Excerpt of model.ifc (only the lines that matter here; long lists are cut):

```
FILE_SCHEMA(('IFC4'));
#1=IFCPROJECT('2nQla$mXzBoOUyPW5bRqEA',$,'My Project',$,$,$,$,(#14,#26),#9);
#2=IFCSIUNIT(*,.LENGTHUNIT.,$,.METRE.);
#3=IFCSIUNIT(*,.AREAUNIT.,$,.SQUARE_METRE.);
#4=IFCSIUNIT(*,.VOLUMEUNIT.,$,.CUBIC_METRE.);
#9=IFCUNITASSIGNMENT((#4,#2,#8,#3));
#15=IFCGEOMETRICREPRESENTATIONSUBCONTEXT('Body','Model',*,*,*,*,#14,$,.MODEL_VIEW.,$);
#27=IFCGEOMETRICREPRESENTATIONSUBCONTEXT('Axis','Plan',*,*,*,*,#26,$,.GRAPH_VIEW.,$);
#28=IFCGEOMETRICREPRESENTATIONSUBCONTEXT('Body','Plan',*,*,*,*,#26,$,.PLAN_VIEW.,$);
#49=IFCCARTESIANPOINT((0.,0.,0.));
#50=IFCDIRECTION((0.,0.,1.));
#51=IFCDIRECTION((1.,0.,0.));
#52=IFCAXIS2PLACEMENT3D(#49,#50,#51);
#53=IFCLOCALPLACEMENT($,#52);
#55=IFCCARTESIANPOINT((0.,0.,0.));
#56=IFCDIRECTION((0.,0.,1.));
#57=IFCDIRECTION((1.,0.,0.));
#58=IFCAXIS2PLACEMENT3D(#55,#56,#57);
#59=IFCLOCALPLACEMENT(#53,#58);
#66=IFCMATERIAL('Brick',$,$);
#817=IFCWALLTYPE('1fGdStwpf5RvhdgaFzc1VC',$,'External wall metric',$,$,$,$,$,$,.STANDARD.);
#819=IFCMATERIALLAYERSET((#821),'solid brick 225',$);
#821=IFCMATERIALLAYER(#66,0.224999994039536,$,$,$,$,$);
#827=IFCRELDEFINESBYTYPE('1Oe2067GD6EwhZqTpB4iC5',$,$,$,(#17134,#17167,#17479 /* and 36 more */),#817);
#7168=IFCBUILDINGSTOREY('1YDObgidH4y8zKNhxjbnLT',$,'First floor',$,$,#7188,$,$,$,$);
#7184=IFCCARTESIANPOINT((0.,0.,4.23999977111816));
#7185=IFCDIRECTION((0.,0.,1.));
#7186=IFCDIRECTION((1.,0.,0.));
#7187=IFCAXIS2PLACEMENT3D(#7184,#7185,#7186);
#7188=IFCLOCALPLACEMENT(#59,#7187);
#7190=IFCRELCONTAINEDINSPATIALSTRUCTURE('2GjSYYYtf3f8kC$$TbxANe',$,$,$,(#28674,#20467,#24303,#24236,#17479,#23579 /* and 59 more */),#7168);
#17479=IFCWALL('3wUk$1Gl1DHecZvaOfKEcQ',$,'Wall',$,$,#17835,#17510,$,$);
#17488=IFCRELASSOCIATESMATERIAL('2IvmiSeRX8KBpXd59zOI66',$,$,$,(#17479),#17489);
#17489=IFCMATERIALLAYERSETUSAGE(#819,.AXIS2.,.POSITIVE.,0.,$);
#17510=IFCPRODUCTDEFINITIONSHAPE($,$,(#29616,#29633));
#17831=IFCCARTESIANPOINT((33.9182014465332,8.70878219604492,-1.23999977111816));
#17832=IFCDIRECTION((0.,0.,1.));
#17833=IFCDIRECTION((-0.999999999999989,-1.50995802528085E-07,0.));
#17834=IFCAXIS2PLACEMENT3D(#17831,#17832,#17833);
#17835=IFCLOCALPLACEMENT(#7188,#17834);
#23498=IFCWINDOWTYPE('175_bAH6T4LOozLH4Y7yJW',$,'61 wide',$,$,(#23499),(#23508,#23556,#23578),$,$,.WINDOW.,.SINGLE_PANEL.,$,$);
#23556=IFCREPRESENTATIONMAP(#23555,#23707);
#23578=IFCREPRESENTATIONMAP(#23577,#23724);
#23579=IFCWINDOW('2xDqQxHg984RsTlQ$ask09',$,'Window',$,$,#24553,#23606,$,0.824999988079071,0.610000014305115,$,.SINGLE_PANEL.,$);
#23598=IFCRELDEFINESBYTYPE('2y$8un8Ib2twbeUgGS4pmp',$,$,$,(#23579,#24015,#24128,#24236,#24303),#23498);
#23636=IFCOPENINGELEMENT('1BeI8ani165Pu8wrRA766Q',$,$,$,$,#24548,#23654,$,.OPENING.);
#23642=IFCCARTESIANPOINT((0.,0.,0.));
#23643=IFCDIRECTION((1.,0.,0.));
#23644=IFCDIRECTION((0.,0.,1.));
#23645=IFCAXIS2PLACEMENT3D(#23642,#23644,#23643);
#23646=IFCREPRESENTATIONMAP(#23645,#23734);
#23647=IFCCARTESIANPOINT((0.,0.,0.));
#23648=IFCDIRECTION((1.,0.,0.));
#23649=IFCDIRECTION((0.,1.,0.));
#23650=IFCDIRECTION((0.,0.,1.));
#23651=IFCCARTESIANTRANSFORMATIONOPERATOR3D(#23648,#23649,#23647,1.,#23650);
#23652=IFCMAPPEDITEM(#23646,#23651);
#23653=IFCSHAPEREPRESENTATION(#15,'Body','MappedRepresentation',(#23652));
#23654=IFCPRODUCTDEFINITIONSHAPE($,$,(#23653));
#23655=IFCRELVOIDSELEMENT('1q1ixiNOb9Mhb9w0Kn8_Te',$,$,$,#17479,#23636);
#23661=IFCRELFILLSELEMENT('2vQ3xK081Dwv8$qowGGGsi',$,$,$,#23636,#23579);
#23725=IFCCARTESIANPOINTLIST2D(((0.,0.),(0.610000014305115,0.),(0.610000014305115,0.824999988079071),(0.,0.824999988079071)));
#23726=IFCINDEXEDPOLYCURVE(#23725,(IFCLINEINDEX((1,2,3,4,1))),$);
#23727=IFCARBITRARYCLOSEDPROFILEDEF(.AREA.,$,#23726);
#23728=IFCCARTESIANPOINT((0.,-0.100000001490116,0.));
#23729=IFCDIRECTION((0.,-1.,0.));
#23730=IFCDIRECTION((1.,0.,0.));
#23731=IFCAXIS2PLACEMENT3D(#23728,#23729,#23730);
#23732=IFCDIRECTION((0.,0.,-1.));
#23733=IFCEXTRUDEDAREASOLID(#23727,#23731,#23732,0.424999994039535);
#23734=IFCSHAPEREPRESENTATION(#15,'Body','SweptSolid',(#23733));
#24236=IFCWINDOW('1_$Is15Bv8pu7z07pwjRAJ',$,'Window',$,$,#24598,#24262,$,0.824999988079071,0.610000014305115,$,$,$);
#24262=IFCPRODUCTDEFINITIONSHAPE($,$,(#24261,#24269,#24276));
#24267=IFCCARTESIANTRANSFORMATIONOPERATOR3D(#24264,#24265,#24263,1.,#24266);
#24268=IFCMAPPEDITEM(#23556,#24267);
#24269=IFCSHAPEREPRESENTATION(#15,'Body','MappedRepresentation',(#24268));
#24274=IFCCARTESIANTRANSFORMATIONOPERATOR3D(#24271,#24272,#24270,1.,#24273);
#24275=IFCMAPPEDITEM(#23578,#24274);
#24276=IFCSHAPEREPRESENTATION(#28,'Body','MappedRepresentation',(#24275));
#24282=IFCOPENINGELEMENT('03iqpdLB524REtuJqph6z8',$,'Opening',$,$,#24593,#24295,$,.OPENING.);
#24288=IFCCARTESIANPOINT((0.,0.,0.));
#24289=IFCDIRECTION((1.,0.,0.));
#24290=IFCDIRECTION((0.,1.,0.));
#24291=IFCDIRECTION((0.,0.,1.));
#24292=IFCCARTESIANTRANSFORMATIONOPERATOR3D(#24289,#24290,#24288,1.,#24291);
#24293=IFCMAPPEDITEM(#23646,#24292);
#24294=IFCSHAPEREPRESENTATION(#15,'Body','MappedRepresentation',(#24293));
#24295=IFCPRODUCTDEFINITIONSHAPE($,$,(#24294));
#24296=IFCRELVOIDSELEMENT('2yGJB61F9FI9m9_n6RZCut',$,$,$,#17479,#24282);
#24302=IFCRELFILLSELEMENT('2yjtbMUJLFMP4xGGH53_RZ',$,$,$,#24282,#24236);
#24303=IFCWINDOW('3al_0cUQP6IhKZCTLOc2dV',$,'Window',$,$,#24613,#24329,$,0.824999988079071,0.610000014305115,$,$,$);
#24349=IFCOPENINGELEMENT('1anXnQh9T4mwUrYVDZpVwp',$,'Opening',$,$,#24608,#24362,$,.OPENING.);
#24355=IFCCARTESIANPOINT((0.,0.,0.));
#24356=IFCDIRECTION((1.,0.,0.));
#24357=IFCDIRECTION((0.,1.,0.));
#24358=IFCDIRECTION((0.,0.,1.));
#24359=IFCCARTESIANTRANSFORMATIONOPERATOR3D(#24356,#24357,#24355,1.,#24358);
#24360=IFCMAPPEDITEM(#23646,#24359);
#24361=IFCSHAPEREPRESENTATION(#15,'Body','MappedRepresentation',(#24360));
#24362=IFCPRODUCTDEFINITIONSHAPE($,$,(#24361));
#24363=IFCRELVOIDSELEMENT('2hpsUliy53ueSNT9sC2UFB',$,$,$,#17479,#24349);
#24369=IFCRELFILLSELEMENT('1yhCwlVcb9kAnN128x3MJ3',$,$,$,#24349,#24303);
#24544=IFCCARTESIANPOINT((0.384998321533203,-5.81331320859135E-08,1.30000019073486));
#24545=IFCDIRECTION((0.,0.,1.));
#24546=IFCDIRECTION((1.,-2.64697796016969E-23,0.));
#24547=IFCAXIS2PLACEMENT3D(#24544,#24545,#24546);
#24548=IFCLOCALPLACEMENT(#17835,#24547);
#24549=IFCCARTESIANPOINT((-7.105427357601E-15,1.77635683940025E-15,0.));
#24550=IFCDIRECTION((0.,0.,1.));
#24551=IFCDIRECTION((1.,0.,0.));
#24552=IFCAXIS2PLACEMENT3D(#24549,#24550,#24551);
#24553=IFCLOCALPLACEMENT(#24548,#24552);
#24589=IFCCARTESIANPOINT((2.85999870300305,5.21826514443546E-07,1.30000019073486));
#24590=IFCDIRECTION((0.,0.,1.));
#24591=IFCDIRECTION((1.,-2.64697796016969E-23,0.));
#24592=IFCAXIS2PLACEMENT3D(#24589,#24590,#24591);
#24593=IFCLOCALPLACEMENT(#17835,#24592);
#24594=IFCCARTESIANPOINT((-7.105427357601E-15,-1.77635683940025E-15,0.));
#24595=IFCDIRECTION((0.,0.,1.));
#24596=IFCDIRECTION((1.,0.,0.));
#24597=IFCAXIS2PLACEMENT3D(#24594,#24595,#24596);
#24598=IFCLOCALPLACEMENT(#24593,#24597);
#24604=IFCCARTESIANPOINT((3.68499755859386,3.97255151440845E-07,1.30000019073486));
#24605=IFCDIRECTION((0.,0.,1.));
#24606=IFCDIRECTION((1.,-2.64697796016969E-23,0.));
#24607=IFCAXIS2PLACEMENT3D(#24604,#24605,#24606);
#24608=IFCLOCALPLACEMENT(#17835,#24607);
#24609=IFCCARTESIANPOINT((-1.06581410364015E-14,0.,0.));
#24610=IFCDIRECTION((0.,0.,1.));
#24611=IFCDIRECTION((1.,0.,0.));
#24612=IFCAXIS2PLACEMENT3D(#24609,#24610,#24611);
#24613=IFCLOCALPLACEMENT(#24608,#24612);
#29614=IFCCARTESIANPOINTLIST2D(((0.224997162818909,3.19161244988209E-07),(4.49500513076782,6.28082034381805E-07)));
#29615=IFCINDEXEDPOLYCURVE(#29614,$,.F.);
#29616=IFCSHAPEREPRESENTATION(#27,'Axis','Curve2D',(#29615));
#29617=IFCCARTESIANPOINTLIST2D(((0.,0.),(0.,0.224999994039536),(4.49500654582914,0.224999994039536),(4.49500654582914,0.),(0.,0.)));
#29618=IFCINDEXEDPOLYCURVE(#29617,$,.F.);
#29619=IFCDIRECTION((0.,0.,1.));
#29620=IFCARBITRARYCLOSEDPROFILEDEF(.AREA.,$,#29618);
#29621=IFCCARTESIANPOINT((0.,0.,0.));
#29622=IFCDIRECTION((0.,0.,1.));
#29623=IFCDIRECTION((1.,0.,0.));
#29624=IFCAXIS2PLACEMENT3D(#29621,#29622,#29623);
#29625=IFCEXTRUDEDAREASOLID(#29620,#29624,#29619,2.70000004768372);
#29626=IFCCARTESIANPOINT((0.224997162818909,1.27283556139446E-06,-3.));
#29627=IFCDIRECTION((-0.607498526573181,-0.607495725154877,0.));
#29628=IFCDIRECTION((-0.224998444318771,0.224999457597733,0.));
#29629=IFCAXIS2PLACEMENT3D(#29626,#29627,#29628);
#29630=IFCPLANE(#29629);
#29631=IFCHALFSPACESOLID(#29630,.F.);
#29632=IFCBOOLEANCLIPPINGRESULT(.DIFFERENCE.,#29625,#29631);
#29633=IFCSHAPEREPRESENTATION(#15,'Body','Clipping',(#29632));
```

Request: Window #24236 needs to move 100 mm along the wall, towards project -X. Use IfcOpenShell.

```python
import ifcopenshell
import ifcopenshell.api.geometry
import ifcopenshell.util.placement

model = ifcopenshell.open("model.ifc")

window = model.by_guid("1_$Is15Bv8pu7z07pwjRAJ")
opening = window.FillsVoids[0].RelatingOpeningElement
wall = opening.VoidsElements[0].RelatingBuildingElement

wall_matrix = ifcopenshell.util.placement.get_local_placement(wall.ObjectPlacement)
shift = wall_matrix[:3, 0] * 0.1
before = ifcopenshell.util.placement.get_local_placement(window.ObjectPlacement)[:3, 3].copy()

# The window is placed relative to its opening, so it follows when the opening moves.
matrix = ifcopenshell.util.placement.get_local_placement(opening.ObjectPlacement)
matrix[:3, 3] += shift
ifcopenshell.api.geometry.edit_object_placement(
    model, product=opening, matrix=matrix, is_si=False, should_transform_children=True
)

after = ifcopenshell.util.placement.get_local_placement(window.ObjectPlacement)[:3, 3]
print("window moved by", (after - before).round(3) + 0.0)

model.write("model_v2.ifc")
```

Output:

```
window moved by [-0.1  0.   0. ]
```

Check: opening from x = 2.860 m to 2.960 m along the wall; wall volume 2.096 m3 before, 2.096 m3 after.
